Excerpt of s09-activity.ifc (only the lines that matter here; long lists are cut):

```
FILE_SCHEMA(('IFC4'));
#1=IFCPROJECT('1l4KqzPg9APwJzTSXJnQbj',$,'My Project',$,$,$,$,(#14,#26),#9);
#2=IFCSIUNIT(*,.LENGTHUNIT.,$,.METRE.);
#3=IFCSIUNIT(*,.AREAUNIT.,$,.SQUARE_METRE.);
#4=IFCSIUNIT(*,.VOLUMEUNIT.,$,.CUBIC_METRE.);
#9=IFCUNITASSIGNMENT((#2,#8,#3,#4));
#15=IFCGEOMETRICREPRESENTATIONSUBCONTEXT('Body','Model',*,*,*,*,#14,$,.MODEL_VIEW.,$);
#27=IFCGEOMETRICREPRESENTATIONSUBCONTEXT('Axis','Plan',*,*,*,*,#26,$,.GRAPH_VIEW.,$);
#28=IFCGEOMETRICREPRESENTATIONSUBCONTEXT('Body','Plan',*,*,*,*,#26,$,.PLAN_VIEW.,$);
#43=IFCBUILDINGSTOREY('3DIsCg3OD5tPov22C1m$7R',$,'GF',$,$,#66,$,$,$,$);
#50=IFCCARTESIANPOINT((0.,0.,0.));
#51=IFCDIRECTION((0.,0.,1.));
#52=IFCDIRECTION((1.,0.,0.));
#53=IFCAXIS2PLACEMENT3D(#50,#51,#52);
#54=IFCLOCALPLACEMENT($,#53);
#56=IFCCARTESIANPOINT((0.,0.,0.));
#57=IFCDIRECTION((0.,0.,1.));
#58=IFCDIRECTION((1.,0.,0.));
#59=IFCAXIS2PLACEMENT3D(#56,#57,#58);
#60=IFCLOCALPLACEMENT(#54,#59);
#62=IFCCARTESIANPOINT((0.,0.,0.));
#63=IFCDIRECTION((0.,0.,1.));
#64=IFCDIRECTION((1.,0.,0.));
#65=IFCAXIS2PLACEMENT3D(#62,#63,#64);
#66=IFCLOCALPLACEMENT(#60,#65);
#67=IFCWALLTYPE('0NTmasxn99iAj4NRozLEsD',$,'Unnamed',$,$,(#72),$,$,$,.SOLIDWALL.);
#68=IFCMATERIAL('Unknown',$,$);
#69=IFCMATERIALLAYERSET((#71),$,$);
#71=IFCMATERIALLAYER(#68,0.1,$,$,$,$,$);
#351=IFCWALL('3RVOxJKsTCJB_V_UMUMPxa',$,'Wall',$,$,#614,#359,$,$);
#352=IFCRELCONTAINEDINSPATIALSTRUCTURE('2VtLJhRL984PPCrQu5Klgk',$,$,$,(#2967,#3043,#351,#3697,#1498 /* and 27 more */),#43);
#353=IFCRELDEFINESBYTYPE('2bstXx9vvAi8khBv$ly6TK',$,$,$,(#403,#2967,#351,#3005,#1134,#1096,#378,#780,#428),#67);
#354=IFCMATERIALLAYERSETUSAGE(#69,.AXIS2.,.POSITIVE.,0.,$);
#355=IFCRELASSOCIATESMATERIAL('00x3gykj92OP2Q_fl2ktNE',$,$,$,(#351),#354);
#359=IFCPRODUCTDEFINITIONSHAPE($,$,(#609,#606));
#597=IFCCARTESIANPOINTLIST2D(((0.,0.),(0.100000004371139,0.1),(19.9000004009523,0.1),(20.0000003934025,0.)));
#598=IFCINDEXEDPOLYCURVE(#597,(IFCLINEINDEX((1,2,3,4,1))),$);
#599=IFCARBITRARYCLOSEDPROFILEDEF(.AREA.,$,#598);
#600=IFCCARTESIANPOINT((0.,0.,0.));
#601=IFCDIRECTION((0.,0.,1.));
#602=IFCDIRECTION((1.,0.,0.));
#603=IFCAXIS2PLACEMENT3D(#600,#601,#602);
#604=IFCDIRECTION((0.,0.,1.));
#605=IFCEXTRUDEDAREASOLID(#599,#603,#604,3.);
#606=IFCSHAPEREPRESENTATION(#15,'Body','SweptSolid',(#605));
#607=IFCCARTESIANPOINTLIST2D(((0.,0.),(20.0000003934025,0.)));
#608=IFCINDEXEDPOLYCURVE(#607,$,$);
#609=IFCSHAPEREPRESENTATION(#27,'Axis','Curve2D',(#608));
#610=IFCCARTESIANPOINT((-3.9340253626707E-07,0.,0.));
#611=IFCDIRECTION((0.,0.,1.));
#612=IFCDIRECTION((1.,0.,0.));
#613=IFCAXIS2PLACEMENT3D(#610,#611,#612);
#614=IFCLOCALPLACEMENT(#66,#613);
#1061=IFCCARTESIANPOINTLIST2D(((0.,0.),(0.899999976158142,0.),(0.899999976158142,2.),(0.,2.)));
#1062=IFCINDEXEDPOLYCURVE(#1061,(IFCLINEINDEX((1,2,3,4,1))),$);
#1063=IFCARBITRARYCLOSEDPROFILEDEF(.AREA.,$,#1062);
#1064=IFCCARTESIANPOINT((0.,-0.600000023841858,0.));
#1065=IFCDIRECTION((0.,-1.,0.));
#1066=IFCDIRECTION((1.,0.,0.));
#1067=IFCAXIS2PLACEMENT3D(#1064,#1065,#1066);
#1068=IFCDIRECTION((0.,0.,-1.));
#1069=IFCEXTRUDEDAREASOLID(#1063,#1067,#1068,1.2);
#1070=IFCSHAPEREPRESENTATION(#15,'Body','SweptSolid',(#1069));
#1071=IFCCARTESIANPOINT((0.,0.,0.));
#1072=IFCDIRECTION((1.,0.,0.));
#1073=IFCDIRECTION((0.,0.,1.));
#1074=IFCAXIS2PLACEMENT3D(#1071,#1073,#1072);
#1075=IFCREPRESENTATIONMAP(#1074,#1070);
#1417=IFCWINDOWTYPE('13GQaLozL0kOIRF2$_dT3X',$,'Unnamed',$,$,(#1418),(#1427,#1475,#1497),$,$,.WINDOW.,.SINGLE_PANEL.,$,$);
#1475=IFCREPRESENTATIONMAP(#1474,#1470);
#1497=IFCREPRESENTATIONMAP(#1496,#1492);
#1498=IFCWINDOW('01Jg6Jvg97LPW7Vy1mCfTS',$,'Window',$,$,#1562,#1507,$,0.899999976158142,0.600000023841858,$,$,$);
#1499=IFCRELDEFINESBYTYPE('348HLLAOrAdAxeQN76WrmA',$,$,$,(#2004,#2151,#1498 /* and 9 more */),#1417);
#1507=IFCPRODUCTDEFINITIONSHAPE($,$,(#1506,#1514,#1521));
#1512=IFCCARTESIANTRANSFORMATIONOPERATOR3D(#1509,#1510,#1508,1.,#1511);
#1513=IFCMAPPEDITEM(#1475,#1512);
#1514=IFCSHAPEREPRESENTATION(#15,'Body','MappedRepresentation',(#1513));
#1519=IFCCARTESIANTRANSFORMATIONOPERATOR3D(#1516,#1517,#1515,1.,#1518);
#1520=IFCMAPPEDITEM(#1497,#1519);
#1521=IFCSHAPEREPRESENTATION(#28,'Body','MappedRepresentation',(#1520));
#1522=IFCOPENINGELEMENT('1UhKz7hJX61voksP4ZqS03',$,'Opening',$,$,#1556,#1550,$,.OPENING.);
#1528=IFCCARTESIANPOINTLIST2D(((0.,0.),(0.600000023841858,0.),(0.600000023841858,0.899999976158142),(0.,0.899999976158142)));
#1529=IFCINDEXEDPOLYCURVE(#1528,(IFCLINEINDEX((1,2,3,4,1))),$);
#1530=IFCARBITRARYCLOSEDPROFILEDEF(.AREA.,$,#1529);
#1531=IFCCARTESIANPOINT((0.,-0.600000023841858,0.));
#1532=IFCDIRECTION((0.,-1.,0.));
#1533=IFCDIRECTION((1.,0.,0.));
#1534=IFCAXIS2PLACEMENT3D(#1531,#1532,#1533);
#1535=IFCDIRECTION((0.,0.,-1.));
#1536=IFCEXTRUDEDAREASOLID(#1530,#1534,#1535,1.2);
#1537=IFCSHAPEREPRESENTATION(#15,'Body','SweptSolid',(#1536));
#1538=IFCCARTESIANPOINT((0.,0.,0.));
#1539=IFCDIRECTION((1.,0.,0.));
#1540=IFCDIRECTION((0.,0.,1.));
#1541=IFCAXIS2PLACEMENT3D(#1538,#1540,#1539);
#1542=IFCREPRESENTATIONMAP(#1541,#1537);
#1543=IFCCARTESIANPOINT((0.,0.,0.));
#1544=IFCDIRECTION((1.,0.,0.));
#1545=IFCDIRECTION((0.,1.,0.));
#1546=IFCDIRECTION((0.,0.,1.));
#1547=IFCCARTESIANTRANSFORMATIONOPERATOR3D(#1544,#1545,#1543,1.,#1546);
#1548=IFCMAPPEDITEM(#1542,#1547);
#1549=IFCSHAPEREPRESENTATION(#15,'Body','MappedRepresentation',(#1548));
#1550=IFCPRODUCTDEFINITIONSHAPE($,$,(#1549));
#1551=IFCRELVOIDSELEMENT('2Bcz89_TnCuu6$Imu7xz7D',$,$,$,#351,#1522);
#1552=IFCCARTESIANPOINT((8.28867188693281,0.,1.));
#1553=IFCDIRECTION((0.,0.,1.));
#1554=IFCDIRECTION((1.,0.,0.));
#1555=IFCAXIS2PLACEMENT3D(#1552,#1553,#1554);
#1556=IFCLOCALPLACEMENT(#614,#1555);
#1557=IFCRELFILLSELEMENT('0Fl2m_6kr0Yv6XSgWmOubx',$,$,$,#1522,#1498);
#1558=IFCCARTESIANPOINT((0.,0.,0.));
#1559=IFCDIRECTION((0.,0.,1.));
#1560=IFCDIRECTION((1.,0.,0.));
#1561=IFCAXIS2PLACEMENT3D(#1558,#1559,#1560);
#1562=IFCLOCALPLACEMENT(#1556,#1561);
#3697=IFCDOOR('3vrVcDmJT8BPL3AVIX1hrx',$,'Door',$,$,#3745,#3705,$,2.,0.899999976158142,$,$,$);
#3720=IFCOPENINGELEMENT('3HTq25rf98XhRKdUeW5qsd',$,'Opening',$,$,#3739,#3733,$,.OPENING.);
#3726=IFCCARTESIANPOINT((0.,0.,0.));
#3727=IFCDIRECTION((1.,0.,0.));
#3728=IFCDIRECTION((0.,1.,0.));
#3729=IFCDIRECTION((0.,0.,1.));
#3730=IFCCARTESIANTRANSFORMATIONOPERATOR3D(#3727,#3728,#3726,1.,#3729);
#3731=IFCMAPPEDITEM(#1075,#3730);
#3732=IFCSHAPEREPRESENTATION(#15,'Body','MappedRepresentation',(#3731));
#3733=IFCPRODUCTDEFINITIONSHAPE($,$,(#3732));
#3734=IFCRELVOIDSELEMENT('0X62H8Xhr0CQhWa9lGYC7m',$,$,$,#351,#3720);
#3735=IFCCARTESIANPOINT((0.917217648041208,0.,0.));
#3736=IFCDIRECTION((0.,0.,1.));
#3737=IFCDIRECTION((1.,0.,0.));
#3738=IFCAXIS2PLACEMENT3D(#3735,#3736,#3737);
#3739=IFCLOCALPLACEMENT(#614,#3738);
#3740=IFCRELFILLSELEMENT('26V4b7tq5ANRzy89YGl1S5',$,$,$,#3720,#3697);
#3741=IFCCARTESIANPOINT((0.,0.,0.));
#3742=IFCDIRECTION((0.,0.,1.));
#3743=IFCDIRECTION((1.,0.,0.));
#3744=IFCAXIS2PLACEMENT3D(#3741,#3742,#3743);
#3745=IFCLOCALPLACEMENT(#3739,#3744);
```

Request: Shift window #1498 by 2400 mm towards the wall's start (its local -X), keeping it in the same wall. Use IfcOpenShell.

```python
import ifcopenshell
import ifcopenshell.api.geometry
import ifcopenshell.util.placement

model = ifcopenshell.open("s09-activity.ifc")

window = model.by_guid("01Jg6Jvg97LPW7Vy1mCfTS")
opening = window.FillsVoids[0].RelatingOpeningElement
wall = opening.VoidsElements[0].RelatingBuildingElement

wall_matrix = ifcopenshell.util.placement.get_local_placement(wall.ObjectPlacement)
shift = wall_matrix[:3, 0] * -2.4
before = ifcopenshell.util.placement.get_local_placement(window.ObjectPlacement)[:3, 3].copy()

# The window is placed relative to its opening, so it follows when the opening moves.
matrix = ifcopenshell.util.placement.get_local_placement(opening.ObjectPlacement)
matrix[:3, 3] += shift
ifcopenshell.api.geometry.edit_object_placement(
    model, product=opening, matrix=matrix, is_si=False, should_transform_children=True
)

after = ifcopenshell.util.placement.get_local_placement(window.ObjectPlacement)[:3, 3]
print("window moved by", (after - before).round(3) + 0.0)

model.write("s09-activity-out.ifc")
```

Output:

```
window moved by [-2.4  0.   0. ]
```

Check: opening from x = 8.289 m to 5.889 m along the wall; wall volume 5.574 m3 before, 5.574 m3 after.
